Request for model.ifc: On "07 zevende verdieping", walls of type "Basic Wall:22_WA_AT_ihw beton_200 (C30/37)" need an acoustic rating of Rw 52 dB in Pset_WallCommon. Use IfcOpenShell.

First a look at what the model holds.

```python
import ifcopenshell
import ifcopenshell.util.element

model = ifcopenshell.open("model.ifc")
print(model.schema)
storey = next(s for s in model.by_type("IfcBuildingStorey") if s.Name == "07 zevende verdieping")
walls = [e for e in ifcopenshell.util.element.get_decomposition(storey) if e.is_a("IfcWall")]
seen = {}
for e in walls:
    element_type = ifcopenshell.util.element.get_type(e)
    key = (element_type.Name if element_type != e and element_type else None, ifcopenshell.util.element.get_pset(e, "Pset_WallCommon", "AcousticRating"))
    seen[key] = seen.get(key, 0) + 1
for (name, value), count in sorted(seen.items(), key=str):
    print(count, "x", name, "|", value)
```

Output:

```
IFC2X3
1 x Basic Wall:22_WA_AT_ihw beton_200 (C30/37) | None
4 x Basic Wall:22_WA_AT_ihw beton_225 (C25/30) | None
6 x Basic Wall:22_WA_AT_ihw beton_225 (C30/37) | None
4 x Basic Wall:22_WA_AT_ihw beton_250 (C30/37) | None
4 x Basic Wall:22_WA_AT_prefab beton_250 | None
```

```python
import ifcopenshell
import ifcopenshell.api.pset
import ifcopenshell.util.element

model = ifcopenshell.open("model.ifc")

storey = next(s for s in model.by_type("IfcBuildingStorey") if s.Name == "07 zevende verdieping")
walls = [e for e in ifcopenshell.util.element.get_decomposition(storey) if e.is_a("IfcWall")]

count = 0
for e in walls:
    element_type = ifcopenshell.util.element.get_type(e)
    if element_type in (None, e) or element_type.Name != "Basic Wall:22_WA_AT_ihw beton_200 (C30/37)":
        continue
    # add_pset returns the element's existing set when there is one.
    pset = ifcopenshell.api.pset.add_pset(model, product=e, name="Pset_WallCommon")
    ifcopenshell.api.pset.edit_pset(model, pset=pset, properties={"AcousticRating": "Rw 52 dB"})
    count += 1

print(count, "walls updated")

model.write("model-out.ifc")
```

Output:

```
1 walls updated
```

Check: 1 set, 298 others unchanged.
